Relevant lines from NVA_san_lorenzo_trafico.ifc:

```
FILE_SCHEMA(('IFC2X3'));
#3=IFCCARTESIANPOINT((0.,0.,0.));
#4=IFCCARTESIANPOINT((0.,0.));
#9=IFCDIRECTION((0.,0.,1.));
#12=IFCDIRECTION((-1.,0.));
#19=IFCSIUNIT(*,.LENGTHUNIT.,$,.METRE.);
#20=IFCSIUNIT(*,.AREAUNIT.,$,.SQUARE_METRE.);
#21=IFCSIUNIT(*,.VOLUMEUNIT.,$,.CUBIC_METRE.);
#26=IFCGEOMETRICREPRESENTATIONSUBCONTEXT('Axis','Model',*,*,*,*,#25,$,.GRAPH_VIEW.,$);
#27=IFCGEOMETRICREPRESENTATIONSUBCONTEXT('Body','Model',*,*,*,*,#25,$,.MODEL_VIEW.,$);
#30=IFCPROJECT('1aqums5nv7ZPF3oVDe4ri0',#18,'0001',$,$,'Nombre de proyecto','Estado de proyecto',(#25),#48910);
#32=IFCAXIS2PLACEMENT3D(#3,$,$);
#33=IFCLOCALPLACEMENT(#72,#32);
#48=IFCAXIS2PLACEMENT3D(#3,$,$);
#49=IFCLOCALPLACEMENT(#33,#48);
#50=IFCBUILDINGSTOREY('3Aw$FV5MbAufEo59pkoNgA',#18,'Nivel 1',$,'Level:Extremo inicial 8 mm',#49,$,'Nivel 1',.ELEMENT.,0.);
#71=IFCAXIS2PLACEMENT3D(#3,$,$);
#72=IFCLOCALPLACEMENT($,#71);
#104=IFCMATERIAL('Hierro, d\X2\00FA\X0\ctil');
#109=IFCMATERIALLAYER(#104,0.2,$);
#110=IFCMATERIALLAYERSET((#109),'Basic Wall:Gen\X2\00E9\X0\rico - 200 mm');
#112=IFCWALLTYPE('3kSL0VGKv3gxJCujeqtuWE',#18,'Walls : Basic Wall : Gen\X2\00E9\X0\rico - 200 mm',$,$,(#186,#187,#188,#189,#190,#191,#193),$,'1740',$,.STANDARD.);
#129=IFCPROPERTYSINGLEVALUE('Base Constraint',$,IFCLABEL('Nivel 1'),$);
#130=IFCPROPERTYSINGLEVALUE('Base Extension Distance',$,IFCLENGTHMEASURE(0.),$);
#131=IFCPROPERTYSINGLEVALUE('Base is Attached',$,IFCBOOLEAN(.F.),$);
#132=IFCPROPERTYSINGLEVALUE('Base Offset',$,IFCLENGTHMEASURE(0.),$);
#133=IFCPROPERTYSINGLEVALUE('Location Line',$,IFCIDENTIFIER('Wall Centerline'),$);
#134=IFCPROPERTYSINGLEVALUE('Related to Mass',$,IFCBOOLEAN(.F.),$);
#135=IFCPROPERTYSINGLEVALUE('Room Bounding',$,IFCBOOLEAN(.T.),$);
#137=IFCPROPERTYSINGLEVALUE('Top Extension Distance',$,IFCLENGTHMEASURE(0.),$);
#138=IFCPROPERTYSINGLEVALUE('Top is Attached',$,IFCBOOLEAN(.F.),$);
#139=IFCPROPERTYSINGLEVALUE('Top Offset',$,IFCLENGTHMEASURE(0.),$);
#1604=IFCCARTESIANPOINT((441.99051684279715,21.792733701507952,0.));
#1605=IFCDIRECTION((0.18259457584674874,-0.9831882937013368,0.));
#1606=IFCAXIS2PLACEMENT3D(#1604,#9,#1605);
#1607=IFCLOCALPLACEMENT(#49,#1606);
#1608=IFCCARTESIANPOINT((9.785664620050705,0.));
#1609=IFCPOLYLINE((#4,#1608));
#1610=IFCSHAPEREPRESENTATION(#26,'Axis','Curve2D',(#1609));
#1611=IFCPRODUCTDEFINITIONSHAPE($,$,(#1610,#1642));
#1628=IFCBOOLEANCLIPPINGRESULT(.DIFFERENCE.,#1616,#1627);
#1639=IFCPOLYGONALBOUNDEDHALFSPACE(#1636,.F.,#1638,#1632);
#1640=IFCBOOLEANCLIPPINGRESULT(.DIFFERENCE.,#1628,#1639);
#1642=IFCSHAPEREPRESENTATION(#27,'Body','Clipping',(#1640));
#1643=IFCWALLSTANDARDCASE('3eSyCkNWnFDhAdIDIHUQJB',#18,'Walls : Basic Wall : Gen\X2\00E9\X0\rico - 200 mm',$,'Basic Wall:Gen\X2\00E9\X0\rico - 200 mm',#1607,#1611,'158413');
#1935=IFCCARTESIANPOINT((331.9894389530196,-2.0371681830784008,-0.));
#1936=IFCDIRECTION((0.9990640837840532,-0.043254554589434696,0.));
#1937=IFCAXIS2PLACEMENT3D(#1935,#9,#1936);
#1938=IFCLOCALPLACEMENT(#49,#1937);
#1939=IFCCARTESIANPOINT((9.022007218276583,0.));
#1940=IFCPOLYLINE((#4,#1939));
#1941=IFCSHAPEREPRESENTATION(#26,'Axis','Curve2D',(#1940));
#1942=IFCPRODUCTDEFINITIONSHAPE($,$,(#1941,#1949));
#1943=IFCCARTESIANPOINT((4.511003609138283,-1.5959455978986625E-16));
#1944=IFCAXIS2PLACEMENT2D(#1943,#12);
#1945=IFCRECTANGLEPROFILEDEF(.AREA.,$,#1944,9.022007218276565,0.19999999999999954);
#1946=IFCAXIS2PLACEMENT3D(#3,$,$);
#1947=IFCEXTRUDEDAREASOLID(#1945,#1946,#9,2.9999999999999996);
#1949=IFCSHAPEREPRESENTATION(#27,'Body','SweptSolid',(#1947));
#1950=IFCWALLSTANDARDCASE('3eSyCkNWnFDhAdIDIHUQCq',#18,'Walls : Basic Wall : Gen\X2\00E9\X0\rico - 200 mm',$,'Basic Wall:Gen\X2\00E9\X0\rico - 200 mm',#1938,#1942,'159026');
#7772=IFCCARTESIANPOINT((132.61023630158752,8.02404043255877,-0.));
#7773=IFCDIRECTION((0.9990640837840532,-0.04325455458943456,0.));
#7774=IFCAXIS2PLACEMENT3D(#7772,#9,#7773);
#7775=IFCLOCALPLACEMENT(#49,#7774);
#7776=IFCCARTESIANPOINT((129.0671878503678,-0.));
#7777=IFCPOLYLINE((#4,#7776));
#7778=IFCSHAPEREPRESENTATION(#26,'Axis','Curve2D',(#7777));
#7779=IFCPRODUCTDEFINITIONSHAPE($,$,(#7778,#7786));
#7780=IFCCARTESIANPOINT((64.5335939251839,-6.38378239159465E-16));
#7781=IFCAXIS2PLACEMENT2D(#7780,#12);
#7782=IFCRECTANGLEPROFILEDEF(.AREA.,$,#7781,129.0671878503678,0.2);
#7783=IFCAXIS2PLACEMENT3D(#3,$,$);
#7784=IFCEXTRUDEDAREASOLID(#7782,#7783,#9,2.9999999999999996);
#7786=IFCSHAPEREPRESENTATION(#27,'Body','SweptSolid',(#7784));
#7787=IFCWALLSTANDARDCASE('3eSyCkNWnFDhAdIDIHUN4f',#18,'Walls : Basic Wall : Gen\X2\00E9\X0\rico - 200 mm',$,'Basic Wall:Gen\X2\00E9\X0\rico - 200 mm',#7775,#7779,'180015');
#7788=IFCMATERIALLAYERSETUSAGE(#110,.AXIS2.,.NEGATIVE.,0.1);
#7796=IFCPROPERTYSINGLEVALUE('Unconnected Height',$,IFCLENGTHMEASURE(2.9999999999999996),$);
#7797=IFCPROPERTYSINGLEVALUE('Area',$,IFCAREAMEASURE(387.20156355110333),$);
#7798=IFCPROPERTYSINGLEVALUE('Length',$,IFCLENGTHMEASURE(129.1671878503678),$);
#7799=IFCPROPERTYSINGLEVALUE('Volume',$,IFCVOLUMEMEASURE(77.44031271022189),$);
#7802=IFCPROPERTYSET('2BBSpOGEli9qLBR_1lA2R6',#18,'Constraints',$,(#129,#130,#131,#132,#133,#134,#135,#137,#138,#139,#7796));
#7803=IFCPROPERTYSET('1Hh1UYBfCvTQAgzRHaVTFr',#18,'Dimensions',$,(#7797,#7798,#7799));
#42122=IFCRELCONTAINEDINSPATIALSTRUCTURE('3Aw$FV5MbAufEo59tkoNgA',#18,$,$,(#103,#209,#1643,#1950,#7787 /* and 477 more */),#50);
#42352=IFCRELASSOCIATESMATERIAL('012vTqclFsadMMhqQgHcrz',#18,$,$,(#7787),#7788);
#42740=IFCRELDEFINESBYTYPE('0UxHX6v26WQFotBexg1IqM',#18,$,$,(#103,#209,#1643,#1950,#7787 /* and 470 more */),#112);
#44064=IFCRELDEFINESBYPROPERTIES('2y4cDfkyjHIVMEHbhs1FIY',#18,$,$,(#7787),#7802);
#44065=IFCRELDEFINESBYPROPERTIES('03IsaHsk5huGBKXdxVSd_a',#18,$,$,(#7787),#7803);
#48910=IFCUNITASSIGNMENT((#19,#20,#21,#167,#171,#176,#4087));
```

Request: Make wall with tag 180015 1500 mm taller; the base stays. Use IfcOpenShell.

```python
import ifcopenshell
import ifcopenshell.api.pset
import ifcopenshell.geom
import ifcopenshell.util.element
import ifcopenshell.util.representation
import ifcopenshell.util.shape
import ifcopenshell.util.unit

model = ifcopenshell.open("NVA_san_lorenzo_trafico.ifc")
area_scale = ifcopenshell.util.unit.calculate_unit_scale(model, "AREAUNIT")
volume_scale = ifcopenshell.util.unit.calculate_unit_scale(model, "VOLUMEUNIT")
settings = ifcopenshell.geom.settings()


def volume(element):
    """Net volume in cubic metres, openings subtracted."""
    shape = ifcopenshell.geom.create_shape(settings, element)
    return ifcopenshell.util.shape.get_volume(shape.geometry)


wall = model.by_guid("3eSyCkNWnFDhAdIDIHUN4f")
before = volume(wall)

body = ifcopenshell.util.representation.get_representation(wall, "Model", "Body")
solid = body.Items[0]
old_height = solid.Depth
solid.Depth += 1.5
after = volume(wall)
thickness = 0.2  # wall thickness in metres

# Update the stored height, areas and volumes.
pset = model.by_id(ifcopenshell.util.element.get_pset(wall, "Constraints", should_inherit=False)["id"])
ifcopenshell.api.pset.edit_pset(model, pset=pset, properties={
    "Unconnected Height": model.create_entity("IfcLengthMeasure", solid.Depth),
})
pset = model.by_id(ifcopenshell.util.element.get_pset(wall, "Dimensions", should_inherit=False)["id"])
ifcopenshell.api.pset.edit_pset(model, pset=pset, properties={
    "Area": model.create_entity("IfcAreaMeasure", after / thickness / area_scale),
    "Volume": model.create_entity("IfcVolumeMeasure", after / volume_scale),
})

print(f"height {old_height:g} -> {solid.Depth:g}, volume {before:.3f} -> {after:.3f} m3")

model.write("NVA_san_lorenzo_trafico_v2.ifc")
```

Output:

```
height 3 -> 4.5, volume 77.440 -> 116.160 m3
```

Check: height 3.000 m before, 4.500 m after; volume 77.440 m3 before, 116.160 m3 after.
